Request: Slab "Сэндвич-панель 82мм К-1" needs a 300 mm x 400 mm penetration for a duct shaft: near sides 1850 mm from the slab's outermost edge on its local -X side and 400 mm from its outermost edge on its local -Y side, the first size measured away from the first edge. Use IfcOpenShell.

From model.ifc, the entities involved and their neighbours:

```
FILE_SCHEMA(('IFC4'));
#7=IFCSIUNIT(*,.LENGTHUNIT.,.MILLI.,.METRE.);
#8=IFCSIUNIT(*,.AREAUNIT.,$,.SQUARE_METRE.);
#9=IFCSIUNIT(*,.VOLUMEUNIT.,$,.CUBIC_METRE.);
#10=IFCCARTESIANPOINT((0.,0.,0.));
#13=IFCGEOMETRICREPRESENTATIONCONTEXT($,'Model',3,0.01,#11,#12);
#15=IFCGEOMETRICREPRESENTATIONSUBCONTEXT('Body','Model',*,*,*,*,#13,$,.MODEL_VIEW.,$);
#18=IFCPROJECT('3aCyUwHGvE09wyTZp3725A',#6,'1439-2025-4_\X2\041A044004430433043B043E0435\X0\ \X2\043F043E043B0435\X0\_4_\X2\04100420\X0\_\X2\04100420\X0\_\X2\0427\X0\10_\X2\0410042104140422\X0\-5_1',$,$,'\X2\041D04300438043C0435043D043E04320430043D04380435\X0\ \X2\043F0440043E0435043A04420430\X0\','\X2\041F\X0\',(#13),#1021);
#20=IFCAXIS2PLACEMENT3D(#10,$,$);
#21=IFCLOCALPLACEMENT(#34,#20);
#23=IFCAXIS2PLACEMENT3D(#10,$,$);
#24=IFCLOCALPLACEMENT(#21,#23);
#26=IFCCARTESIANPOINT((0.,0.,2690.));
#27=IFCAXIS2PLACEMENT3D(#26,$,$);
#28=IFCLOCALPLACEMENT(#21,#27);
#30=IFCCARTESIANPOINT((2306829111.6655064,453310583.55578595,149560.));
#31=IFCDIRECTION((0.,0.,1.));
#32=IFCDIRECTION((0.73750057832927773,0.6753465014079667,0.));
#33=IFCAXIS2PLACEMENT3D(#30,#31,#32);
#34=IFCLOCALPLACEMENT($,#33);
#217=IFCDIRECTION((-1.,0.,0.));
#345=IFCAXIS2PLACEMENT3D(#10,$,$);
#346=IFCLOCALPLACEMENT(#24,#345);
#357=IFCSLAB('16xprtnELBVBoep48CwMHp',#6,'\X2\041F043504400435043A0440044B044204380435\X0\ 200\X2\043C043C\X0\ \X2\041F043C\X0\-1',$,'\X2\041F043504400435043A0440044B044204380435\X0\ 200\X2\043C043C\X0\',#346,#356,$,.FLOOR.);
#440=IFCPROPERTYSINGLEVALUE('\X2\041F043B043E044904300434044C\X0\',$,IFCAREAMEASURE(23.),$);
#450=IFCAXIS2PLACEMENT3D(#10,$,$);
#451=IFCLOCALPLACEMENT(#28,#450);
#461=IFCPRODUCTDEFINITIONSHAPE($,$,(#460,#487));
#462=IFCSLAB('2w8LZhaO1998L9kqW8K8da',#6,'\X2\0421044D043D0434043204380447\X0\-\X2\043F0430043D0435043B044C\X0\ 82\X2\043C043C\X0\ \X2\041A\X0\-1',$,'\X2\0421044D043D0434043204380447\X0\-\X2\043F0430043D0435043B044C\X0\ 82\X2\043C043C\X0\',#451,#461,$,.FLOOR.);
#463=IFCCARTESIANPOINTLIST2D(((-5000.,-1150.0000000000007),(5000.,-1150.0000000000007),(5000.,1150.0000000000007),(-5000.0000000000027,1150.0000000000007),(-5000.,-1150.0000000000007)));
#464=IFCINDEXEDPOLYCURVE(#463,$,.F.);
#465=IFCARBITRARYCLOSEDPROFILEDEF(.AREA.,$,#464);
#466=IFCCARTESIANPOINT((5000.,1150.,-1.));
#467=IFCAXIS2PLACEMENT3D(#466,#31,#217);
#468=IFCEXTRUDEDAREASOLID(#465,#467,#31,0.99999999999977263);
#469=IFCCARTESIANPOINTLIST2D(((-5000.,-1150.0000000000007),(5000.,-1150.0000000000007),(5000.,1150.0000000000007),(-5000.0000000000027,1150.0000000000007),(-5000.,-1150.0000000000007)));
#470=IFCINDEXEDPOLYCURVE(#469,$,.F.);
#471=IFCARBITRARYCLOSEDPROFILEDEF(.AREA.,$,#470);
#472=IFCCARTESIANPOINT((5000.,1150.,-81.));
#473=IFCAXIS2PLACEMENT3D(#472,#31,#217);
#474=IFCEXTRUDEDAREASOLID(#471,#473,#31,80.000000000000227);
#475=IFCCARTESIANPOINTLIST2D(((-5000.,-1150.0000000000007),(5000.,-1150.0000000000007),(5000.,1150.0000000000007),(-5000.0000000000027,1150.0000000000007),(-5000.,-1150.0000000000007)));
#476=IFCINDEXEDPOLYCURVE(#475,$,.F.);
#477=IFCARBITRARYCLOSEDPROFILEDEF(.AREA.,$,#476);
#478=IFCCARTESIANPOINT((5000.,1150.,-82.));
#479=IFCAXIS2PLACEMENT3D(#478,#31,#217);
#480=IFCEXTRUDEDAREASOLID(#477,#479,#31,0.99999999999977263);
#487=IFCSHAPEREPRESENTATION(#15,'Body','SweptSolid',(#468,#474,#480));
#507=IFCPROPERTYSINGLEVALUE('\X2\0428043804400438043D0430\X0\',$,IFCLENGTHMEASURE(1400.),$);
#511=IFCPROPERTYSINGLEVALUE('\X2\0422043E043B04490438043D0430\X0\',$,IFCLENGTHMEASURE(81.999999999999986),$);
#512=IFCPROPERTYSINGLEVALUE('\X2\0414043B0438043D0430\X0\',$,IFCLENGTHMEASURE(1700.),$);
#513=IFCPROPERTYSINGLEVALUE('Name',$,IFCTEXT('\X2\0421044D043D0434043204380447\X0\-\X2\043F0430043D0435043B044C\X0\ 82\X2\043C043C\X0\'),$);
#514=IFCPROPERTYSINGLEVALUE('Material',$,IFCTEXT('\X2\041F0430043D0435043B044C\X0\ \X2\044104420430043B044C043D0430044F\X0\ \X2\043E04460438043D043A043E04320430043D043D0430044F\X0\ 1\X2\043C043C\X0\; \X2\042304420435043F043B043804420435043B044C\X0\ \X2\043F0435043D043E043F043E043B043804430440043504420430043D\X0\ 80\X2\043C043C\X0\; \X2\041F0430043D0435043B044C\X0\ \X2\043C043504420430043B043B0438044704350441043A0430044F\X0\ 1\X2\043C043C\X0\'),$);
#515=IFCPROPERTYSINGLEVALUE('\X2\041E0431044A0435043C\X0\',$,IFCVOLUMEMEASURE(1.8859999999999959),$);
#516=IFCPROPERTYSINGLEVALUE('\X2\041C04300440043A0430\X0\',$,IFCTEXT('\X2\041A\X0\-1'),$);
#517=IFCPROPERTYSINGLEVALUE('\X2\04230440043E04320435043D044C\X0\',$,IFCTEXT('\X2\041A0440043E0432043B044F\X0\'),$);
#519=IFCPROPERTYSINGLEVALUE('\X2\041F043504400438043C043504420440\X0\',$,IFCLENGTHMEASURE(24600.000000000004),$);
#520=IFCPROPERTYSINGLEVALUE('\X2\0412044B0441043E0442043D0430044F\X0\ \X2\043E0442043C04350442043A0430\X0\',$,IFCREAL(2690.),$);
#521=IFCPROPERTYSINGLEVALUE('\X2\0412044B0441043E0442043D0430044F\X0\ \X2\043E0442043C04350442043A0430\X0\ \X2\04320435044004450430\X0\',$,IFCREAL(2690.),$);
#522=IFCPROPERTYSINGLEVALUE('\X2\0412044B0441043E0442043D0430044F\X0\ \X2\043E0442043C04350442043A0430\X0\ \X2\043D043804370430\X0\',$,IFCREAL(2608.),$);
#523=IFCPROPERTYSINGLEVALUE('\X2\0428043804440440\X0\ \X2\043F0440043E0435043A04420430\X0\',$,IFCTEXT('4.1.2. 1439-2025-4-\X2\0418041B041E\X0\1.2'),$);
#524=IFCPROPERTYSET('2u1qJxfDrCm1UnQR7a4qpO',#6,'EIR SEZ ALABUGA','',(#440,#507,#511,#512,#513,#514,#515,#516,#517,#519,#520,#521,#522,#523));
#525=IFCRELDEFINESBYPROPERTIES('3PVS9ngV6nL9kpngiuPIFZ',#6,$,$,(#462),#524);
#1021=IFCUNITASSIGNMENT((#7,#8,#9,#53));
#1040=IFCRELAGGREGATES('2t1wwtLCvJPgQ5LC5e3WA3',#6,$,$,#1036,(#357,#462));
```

```python
import numpy as np
import ifcopenshell
import ifcopenshell.api.feature
import ifcopenshell.api.geometry
import ifcopenshell.api.pset
import ifcopenshell.api.root
import ifcopenshell.geom
import ifcopenshell.util.element
import ifcopenshell.util.placement
import ifcopenshell.util.representation
import ifcopenshell.util.shape
import ifcopenshell.util.unit

model = ifcopenshell.open("model.ifc")
unit_scale = ifcopenshell.util.unit.calculate_unit_scale(model)
area_scale = ifcopenshell.util.unit.calculate_unit_scale(model, "AREAUNIT")
volume_scale = ifcopenshell.util.unit.calculate_unit_scale(model, "VOLUMEUNIT")
settings = ifcopenshell.geom.settings()


def volume(element):
    """Net volume in cubic metres, openings subtracted."""
    shape = ifcopenshell.geom.create_shape(settings, element)
    return ifcopenshell.util.shape.get_volume(shape.geometry)


slab = model.by_guid("2w8LZhaO1998L9kqW8K8da")
before = volume(slab)

# Extent in the slab's own axes, in metres. The edges named are its -X and -Y sides.
slab_shape = ifcopenshell.geom.create_shape(settings, slab)
vertices = ifcopenshell.util.shape.get_vertices(slab_shape.geometry)
x_min, y_min, bottom = vertices.min(axis=0)
top = vertices[:, 2].max()

opening = ifcopenshell.api.root.create_entity(model, ifc_class="IfcOpeningElement", name="Duct shaft opening", predefined_type="OPENING")
context = ifcopenshell.util.representation.get_context(model, "Model", "Body", "MODEL_VIEW")
width, depth = 0.3, 0.4
outline = [(0.0, 0.0), (width, 0.0), (width, depth), (0.0, depth), (0.0, 0.0)]
# Overshoot both faces by 50 mm so the cut is clean.
shape = ifcopenshell.api.geometry.add_slab_representation(
    model, context=context, depth=top - bottom + 0.1, polyline=outline
)
ifcopenshell.api.geometry.assign_representation(model, product=opening, representation=shape)

matrix = ifcopenshell.util.placement.get_local_placement(slab.ObjectPlacement)
matrix[:, 3] = matrix @ np.append(np.array([x_min + 1.85, y_min + 0.4, bottom - 0.05]) / unit_scale, 1.0)
ifcopenshell.api.geometry.edit_object_placement(model, product=opening, matrix=matrix, is_si=False)
ifcopenshell.api.feature.add_feature(model, feature=opening, element=slab)

after = volume(slab)

# Update the slab's stored quantities.
pset = model.by_id(ifcopenshell.util.element.get_pset(slab, "EIR SEZ ALABUGA", should_inherit=False)["id"])
ifcopenshell.api.pset.edit_pset(model, pset=pset, properties={
    "Площадь": model.create_entity("IfcAreaMeasure", after / (top - bottom) / area_scale),
    "Объем": model.create_entity("IfcVolumeMeasure", after / volume_scale),
})

print(f"slab volume {before:.3f} -> {after:.3f} m3")

model.write("model-out.ifc")
```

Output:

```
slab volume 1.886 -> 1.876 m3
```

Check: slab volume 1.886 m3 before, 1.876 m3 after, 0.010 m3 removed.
